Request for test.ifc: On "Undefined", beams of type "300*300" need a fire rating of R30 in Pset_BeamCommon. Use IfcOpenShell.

First a look at what the model holds.

```python
import ifcopenshell
import ifcopenshell.util.element

model = ifcopenshell.open("test.ifc")
print(model.schema)
storey = next(s for s in model.by_type("IfcBuildingStorey") if s.Name == "Undefined")
beams = [e for e in ifcopenshell.util.element.get_decomposition(storey) if e.is_a("IfcBeam")]
seen = {}
for e in beams:
    element_type = ifcopenshell.util.element.get_type(e)
    key = (element_type.Name if element_type != e and element_type else None, ifcopenshell.util.element.get_pset(e, "Pset_BeamCommon", "FireRating"))
    seen[key] = seen.get(key, 0) + 1
for (name, value), count in sorted(seen.items(), key=str):
    print(count, "x", name, "|", value)
```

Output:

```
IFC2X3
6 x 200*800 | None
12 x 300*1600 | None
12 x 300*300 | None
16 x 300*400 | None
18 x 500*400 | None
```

```python
import ifcopenshell
import ifcopenshell.api.pset
import ifcopenshell.util.element

model = ifcopenshell.open("test.ifc")

storey = next(s for s in model.by_type("IfcBuildingStorey") if s.Name == "Undefined")
beams = [e for e in ifcopenshell.util.element.get_decomposition(storey) if e.is_a("IfcBeam")]

count = 0
for e in beams:
    element_type = ifcopenshell.util.element.get_type(e)
    if element_type in (None, e) or element_type.Name != "300*300":
        continue
    found = ifcopenshell.util.element.get_pset(e, "Pset_BeamCommon", should_inherit=False)
    if found:
        pset = model.by_id(found["id"])
        if len(ifcopenshell.util.element.get_elements_by_pset(pset)) > 1:
            pset = ifcopenshell.api.pset.unshare_pset(model, products=[e], pset=pset)[0]
    else:
        pset = ifcopenshell.api.pset.add_pset(model, product=e, name="Pset_BeamCommon")
    ifcopenshell.api.pset.edit_pset(model, pset=pset, properties={"FireRating": "R30"})
    count += 1

print(count, "beams updated")

model.write("test_edited.ifc")
```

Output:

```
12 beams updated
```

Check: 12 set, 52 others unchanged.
